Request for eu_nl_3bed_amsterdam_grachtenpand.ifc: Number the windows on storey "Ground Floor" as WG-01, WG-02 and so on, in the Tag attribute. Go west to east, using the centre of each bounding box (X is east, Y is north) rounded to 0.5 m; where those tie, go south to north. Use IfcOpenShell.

First a look at what the model holds.

```python
import ifcopenshell
import ifcopenshell.util.element
import ifcopenshell.util.placement

model = ifcopenshell.open("eu_nl_3bed_amsterdam_grachtenpand.ifc")
print(model.schema)
storey = next(s for s in model.by_type("IfcBuildingStorey") if s.Name == "Ground Floor")
windows = [e for e in ifcopenshell.util.element.get_decomposition(storey) if e.is_a("IfcWindow")]
for e in sorted(windows, key=lambda e: e.id()):
    origin = ifcopenshell.util.placement.get_local_placement(e.ObjectPlacement)[:3, 3]
    print(e.id(), e.Tag, e.Name, origin.round(2) + 0.0, sep=" | ")
```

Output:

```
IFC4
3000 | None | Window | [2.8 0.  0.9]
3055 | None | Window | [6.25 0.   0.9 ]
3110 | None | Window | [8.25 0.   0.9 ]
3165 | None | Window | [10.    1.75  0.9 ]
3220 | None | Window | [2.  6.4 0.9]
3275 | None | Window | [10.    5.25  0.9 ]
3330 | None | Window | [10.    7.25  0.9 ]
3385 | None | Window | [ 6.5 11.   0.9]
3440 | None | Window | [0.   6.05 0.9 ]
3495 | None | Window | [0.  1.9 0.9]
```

```python
import ifcopenshell
import ifcopenshell.geom
import ifcopenshell.util.element
import ifcopenshell.util.shape

model = ifcopenshell.open("eu_nl_3bed_amsterdam_grachtenpand.ifc")
settings = ifcopenshell.geom.settings()
settings.set("use-world-coords", True)


def centre(element):
    shape = ifcopenshell.geom.create_shape(settings, element)
    return ifcopenshell.util.shape.get_bbox_centroid(shape.geometry)


storey = next(s for s in model.by_type("IfcBuildingStorey") if s.Name == "Ground Floor")
windows = [e for e in ifcopenshell.util.element.get_decomposition(storey) if e.is_a("IfcWindow")]

# Insertion points can sit at a corner or the storey origin, so sort by the geometry (in metres).
centres = {e: centre(e) for e in windows}
windows.sort(key=lambda e: (round(centres[e][0] / 0.5), centres[e][1]))

for i, e in enumerate(windows, start=1):
    number = f"WG-{i:02d}"
    e.Tag = number
    print(e.id(), number)

model.write("eu_nl_3bed_amsterdam_grachtenpand_edited.ifc")
```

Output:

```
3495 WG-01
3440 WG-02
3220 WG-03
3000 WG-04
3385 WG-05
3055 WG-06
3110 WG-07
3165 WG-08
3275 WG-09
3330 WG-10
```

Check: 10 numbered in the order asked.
